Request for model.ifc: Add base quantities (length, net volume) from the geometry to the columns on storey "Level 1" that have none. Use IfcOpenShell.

First a look at what the model holds.

```python
import ifcopenshell
import ifcopenshell.util.element
import ifcopenshell.util.unit

model = ifcopenshell.open("model.ifc")
print(model.schema)
for unit_type in ("LENGTHUNIT", "AREAUNIT", "VOLUMEUNIT"):
    print(unit_type, ifcopenshell.util.unit.calculate_unit_scale(model, unit_type))
storey = next(s for s in model.by_type("IfcBuildingStorey") if s.Name == "Level 1")
columns = [e for e in ifcopenshell.util.element.get_decomposition(storey) if e.is_a("IfcColumn")]
for e in sorted(columns, key=lambda e: e.id()):
    print(e.id(), e.is_a(), e.Name, list(ifcopenshell.util.element.get_psets(e, qtos_only=True)), sep=" | ")
```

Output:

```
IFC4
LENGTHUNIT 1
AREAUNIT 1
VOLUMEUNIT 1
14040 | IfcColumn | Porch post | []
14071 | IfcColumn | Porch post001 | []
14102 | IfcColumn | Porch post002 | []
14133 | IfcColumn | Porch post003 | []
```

```python
import ifcopenshell
import ifcopenshell.api.pset
import ifcopenshell.geom
import ifcopenshell.util.element
import ifcopenshell.util.shape
import ifcopenshell.util.unit

model = ifcopenshell.open("model.ifc")
unit_scale = ifcopenshell.util.unit.calculate_unit_scale(model)
volume_scale = ifcopenshell.util.unit.calculate_unit_scale(model, "VOLUMEUNIT")
settings = ifcopenshell.geom.settings()

storey = next(s for s in model.by_type("IfcBuildingStorey") if s.Name == "Level 1")
columns = [e for e in ifcopenshell.util.element.get_decomposition(storey) if e.is_a("IfcColumn")]

for e in sorted(columns, key=lambda e: e.id()):
    if ifcopenshell.util.element.get_psets(e, qtos_only=True, should_inherit=False):
        continue
    # Geometry comes back in metres, in the element's own axes.
    shape = ifcopenshell.geom.create_shape(settings, e)
    values = {
        "Length": ifcopenshell.util.shape.get_z(shape.geometry) / unit_scale,
        "NetVolume": ifcopenshell.util.shape.get_volume(shape.geometry) / volume_scale,
    }
    qto = ifcopenshell.api.pset.add_qto(model, product=e, name="Qto_ColumnBaseQuantities")
    ifcopenshell.api.pset.edit_qto(model, qto=qto, properties=values)
    print(e.id(), {k: round(v, 3) for k, v in values.items()})

model.write("model_updated.ifc")
```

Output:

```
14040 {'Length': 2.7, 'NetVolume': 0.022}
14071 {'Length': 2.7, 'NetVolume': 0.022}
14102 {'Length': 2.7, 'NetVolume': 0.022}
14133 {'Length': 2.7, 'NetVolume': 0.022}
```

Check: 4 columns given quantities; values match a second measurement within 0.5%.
